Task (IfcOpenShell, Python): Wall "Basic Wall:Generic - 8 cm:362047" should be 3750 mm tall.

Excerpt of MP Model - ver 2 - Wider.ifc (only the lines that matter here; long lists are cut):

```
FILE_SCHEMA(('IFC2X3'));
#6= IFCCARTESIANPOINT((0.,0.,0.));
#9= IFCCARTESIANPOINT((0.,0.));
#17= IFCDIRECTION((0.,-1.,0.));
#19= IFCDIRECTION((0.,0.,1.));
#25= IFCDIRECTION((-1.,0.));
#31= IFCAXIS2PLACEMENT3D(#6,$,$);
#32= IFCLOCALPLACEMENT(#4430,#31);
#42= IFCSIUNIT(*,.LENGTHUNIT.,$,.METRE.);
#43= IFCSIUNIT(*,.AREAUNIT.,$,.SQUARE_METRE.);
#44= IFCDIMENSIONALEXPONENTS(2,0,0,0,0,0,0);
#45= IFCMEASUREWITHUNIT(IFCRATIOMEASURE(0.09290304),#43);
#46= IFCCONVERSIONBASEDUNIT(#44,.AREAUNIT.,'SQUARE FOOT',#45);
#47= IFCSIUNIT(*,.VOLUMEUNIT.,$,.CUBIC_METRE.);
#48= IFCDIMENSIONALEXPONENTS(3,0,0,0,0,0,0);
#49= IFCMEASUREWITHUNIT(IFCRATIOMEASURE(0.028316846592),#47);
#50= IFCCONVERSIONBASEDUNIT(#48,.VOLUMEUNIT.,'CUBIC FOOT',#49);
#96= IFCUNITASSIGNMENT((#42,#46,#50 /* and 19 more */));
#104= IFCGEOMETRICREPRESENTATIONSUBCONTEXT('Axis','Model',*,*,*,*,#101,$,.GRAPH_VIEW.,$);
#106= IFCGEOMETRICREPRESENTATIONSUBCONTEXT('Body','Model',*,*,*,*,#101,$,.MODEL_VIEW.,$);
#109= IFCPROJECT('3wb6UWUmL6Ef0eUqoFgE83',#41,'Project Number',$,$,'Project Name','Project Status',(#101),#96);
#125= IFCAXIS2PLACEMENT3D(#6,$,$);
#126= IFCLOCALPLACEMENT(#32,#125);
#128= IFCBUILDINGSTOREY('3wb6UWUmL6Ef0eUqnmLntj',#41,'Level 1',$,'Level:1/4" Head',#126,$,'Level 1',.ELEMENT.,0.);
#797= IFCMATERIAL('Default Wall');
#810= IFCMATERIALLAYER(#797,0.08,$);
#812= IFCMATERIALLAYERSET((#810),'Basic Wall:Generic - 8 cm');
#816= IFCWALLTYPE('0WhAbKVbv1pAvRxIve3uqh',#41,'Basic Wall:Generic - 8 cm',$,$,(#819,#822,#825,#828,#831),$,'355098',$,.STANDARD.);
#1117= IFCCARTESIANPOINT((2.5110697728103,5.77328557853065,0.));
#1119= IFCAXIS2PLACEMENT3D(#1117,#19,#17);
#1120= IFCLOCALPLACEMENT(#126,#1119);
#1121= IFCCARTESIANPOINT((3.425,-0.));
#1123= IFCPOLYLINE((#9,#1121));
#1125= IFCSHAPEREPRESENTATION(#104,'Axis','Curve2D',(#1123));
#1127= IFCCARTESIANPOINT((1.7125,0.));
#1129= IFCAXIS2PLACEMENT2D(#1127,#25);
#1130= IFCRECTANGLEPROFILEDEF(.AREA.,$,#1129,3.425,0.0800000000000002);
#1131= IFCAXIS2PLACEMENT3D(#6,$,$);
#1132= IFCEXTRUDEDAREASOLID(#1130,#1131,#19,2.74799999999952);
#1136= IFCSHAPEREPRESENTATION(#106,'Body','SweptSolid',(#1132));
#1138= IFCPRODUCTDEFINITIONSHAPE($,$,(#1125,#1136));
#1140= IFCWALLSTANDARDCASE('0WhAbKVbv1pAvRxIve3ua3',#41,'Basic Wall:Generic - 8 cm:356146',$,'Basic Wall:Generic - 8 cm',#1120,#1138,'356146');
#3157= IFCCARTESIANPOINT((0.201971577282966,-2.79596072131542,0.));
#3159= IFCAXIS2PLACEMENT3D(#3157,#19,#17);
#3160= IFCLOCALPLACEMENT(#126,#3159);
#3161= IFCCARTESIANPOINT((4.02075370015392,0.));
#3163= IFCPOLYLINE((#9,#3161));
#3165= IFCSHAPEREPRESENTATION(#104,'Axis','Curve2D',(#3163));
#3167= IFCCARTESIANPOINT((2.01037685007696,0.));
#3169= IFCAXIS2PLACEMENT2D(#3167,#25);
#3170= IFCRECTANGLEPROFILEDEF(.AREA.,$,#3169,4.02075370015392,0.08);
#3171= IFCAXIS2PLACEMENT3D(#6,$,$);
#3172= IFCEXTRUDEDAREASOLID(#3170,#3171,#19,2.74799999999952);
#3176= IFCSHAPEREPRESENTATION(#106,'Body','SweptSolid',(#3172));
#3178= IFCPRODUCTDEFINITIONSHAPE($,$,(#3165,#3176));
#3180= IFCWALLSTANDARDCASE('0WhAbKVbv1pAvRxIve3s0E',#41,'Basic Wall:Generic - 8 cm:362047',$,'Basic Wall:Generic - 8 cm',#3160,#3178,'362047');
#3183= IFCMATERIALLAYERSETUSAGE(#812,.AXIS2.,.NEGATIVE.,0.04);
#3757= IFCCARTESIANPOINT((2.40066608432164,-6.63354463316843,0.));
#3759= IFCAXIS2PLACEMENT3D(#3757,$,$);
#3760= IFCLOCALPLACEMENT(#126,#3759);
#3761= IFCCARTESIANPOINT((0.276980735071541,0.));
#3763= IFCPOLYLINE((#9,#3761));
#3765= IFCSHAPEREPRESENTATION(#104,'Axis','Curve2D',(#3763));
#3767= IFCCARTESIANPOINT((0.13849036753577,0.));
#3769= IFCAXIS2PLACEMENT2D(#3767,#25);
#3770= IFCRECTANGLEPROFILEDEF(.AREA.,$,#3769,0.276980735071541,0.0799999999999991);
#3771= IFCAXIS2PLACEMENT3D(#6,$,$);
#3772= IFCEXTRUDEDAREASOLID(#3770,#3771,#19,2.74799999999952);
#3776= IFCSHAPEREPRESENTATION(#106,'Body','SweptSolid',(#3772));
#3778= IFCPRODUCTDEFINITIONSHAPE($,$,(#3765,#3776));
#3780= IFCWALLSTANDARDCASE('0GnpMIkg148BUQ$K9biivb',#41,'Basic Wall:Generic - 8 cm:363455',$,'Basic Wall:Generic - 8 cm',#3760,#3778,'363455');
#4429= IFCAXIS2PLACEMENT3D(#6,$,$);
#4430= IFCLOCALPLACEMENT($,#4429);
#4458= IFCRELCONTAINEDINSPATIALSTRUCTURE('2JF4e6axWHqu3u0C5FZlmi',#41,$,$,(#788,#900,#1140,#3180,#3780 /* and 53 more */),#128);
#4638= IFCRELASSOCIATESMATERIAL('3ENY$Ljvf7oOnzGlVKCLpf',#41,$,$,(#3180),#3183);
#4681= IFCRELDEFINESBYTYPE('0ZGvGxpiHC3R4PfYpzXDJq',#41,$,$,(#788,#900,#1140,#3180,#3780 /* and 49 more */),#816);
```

```python
import ifcopenshell
import ifcopenshell.geom
import ifcopenshell.util.representation
import ifcopenshell.util.shape
import ifcopenshell.util.unit

model = ifcopenshell.open("MP Model - ver 2 - Wider.ifc")
unit_scale = ifcopenshell.util.unit.calculate_unit_scale(model)
settings = ifcopenshell.geom.settings()


def volume(element):
    """Net volume in cubic metres, openings subtracted."""
    shape = ifcopenshell.geom.create_shape(settings, element)
    return ifcopenshell.util.shape.get_volume(shape.geometry)


wall = model.by_guid("0WhAbKVbv1pAvRxIve3s0E")
before = volume(wall)

body = ifcopenshell.util.representation.get_representation(wall, "Model", "Body")
solid = body.Items[0]
old_height = solid.Depth
solid.Depth = 3.75 / unit_scale
after = volume(wall)

print(f"height {old_height:g} -> {solid.Depth:g}, volume {before:.3f} -> {after:.3f} m3")

model.write("MP Model - ver 2 - Wider-out.ifc")
```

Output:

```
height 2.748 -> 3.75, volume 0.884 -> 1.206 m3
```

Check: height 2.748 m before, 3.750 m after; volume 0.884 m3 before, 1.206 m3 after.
